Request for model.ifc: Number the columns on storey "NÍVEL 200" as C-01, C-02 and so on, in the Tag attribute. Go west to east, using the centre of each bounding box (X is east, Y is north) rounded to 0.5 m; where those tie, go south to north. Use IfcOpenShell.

First a look at what the model holds.

```python
import ifcopenshell
import ifcopenshell.util.element
import ifcopenshell.util.placement

model = ifcopenshell.open("model.ifc")
print(model.schema)
storey = next(s for s in model.by_type("IfcBuildingStorey") if s.Name == "NÍVEL 200")
columns = [e for e in ifcopenshell.util.element.get_decomposition(storey) if e.is_a("IfcColumn")]
for e in sorted(columns, key=lambda e: e.id()):
    origin = ifcopenshell.util.placement.get_local_placement(e.ObjectPlacement)[:3, 3]
    print(e.id(), e.Tag, e.Name, origin.round(2) + 0.0, sep=" | ")
```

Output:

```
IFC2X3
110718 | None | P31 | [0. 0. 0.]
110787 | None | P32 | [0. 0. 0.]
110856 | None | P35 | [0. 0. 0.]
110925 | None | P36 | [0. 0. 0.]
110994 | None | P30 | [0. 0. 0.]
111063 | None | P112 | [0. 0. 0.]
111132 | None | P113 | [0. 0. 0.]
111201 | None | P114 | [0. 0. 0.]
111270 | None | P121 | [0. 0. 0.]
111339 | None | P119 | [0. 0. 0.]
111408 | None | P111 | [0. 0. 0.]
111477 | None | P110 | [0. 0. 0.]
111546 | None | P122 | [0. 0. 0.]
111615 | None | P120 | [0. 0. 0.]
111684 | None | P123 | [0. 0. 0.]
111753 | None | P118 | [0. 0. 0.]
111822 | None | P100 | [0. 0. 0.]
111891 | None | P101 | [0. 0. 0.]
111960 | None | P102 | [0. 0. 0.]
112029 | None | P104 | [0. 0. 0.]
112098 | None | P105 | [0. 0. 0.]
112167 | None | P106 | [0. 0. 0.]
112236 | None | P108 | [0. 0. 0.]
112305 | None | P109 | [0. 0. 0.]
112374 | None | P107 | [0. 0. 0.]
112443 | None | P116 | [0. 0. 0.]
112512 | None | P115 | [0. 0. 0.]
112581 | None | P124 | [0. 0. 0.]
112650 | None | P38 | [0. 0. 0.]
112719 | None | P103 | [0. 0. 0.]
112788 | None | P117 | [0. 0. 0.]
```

```python
import ifcopenshell
import ifcopenshell.geom
import ifcopenshell.util.element
import ifcopenshell.util.shape

model = ifcopenshell.open("model.ifc")
settings = ifcopenshell.geom.settings()
settings.set("use-world-coords", True)


def centre(element):
    shape = ifcopenshell.geom.create_shape(settings, element)
    return ifcopenshell.util.shape.get_bbox_centroid(shape.geometry)


storey = next(s for s in model.by_type("IfcBuildingStorey") if s.Name == "NÍVEL 200")
columns = [e for e in ifcopenshell.util.element.get_decomposition(storey) if e.is_a("IfcColumn")]

# Insertion points can sit at a corner or the storey origin, so sort by the geometry (in metres).
centres = {e: centre(e) for e in columns}
columns.sort(key=lambda e: (round(centres[e][0] / 0.5), centres[e][1]))

for i, e in enumerate(columns, start=1):
    number = f"C-{i:02d}"
    e.Tag = number
    print(e.id(), number)

model.write("model_edited.ifc")
```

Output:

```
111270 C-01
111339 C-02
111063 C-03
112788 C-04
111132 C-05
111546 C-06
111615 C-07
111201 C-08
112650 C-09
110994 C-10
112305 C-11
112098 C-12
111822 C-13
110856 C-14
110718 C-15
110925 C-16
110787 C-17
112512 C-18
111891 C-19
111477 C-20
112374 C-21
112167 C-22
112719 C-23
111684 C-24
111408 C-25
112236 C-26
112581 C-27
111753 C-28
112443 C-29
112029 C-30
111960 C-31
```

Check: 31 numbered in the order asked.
